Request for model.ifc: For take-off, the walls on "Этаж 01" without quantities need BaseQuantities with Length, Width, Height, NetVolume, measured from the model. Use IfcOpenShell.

First a look at what the model holds.

```python
import ifcopenshell
import ifcopenshell.util.element
import ifcopenshell.util.unit

model = ifcopenshell.open("model.ifc")
print(model.schema)
for unit_type in ("LENGTHUNIT", "AREAUNIT", "VOLUMEUNIT"):
    print(unit_type, ifcopenshell.util.unit.calculate_unit_scale(model, unit_type))
storey = next(s for s in model.by_type("IfcBuildingStorey") if s.Name == "Этаж 01")
walls = [e for e in ifcopenshell.util.element.get_decomposition(storey) if e.is_a("IfcWall")]
for e in sorted(walls, key=lambda e: e.id()):
    print(e.id(), e.is_a(), e.Name, list(ifcopenshell.util.element.get_psets(e, qtos_only=True)), sep=" | ")
```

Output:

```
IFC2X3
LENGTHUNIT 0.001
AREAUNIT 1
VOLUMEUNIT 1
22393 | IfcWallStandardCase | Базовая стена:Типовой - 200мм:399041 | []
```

```python
import ifcopenshell
import ifcopenshell.api.pset
import ifcopenshell.geom
import ifcopenshell.util.element
import ifcopenshell.util.shape
import ifcopenshell.util.unit

model = ifcopenshell.open("model.ifc")
unit_scale = ifcopenshell.util.unit.calculate_unit_scale(model)
volume_scale = ifcopenshell.util.unit.calculate_unit_scale(model, "VOLUMEUNIT")
settings = ifcopenshell.geom.settings()

storey = next(s for s in model.by_type("IfcBuildingStorey") if s.Name == "Этаж 01")
walls = [e for e in ifcopenshell.util.element.get_decomposition(storey) if e.is_a("IfcWall")]

for e in sorted(walls, key=lambda e: e.id()):
    if ifcopenshell.util.element.get_psets(e, qtos_only=True, should_inherit=False):
        continue
    # Geometry comes back in metres, in the element's own axes.
    shape = ifcopenshell.geom.create_shape(settings, e)
    values = {
        "Length": ifcopenshell.util.shape.get_x(shape.geometry) / unit_scale,
        "Width": ifcopenshell.util.shape.get_y(shape.geometry) / unit_scale,
        "Height": ifcopenshell.util.shape.get_z(shape.geometry) / unit_scale,
        "NetVolume": ifcopenshell.util.shape.get_volume(shape.geometry) / volume_scale,
    }
    qto = ifcopenshell.api.pset.add_qto(model, product=e, name="BaseQuantities")
    ifcopenshell.api.pset.edit_qto(model, qto=qto, properties=values)
    print(e.id(), {k: round(v, 3) for k, v in values.items()})

model.write("model_updated.ifc")
```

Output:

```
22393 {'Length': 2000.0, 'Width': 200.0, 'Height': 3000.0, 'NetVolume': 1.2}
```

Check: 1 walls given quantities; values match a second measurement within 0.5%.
